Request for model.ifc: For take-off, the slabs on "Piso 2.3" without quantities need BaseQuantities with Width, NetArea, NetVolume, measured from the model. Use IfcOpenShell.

First a look at what the model holds.

```python
import ifcopenshell
import ifcopenshell.util.element
import ifcopenshell.util.unit

model = ifcopenshell.open("model.ifc")
print(model.schema)
for unit_type in ("LENGTHUNIT", "AREAUNIT", "VOLUMEUNIT"):
    print(unit_type, ifcopenshell.util.unit.calculate_unit_scale(model, unit_type))
storey = next(s for s in model.by_type("IfcBuildingStorey") if s.Name == "Piso 2.3")
slabs = [e for e in ifcopenshell.util.element.get_decomposition(storey) if e.is_a("IfcSlab")]
for e in sorted(slabs, key=lambda e: e.id()):
    print(e.id(), e.is_a(), e.Name, list(ifcopenshell.util.element.get_psets(e, qtos_only=True)), sep=" | ")
```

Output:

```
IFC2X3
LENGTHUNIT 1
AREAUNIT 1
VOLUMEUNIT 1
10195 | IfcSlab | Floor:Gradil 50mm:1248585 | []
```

```python
import ifcopenshell
import ifcopenshell.api.pset
import ifcopenshell.geom
import ifcopenshell.util.element
import ifcopenshell.util.shape
import ifcopenshell.util.unit

model = ifcopenshell.open("model.ifc")
unit_scale = ifcopenshell.util.unit.calculate_unit_scale(model)
area_scale = ifcopenshell.util.unit.calculate_unit_scale(model, "AREAUNIT")
volume_scale = ifcopenshell.util.unit.calculate_unit_scale(model, "VOLUMEUNIT")
settings = ifcopenshell.geom.settings()

storey = next(s for s in model.by_type("IfcBuildingStorey") if s.Name == "Piso 2.3")
slabs = [e for e in ifcopenshell.util.element.get_decomposition(storey) if e.is_a("IfcSlab")]

for e in sorted(slabs, key=lambda e: e.id()):
    if ifcopenshell.util.element.get_psets(e, qtos_only=True, should_inherit=False):
        continue
    # Geometry comes back in metres, in the element's own axes.
    shape = ifcopenshell.geom.create_shape(settings, e)
    values = {
        "Width": ifcopenshell.util.shape.get_z(shape.geometry) / unit_scale,
        "NetArea": ifcopenshell.util.shape.get_footprint_area(shape.geometry) / area_scale,
        "NetVolume": ifcopenshell.util.shape.get_volume(shape.geometry) / volume_scale,
    }
    qto = ifcopenshell.api.pset.add_qto(model, product=e, name="BaseQuantities")
    ifcopenshell.api.pset.edit_qto(model, qto=qto, properties=values)
    print(e.id(), {k: round(v, 3) for k, v in values.items()})

model.write("model_updated.ifc")
```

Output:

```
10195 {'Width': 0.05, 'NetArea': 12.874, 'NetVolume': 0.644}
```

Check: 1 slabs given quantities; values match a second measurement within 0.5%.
